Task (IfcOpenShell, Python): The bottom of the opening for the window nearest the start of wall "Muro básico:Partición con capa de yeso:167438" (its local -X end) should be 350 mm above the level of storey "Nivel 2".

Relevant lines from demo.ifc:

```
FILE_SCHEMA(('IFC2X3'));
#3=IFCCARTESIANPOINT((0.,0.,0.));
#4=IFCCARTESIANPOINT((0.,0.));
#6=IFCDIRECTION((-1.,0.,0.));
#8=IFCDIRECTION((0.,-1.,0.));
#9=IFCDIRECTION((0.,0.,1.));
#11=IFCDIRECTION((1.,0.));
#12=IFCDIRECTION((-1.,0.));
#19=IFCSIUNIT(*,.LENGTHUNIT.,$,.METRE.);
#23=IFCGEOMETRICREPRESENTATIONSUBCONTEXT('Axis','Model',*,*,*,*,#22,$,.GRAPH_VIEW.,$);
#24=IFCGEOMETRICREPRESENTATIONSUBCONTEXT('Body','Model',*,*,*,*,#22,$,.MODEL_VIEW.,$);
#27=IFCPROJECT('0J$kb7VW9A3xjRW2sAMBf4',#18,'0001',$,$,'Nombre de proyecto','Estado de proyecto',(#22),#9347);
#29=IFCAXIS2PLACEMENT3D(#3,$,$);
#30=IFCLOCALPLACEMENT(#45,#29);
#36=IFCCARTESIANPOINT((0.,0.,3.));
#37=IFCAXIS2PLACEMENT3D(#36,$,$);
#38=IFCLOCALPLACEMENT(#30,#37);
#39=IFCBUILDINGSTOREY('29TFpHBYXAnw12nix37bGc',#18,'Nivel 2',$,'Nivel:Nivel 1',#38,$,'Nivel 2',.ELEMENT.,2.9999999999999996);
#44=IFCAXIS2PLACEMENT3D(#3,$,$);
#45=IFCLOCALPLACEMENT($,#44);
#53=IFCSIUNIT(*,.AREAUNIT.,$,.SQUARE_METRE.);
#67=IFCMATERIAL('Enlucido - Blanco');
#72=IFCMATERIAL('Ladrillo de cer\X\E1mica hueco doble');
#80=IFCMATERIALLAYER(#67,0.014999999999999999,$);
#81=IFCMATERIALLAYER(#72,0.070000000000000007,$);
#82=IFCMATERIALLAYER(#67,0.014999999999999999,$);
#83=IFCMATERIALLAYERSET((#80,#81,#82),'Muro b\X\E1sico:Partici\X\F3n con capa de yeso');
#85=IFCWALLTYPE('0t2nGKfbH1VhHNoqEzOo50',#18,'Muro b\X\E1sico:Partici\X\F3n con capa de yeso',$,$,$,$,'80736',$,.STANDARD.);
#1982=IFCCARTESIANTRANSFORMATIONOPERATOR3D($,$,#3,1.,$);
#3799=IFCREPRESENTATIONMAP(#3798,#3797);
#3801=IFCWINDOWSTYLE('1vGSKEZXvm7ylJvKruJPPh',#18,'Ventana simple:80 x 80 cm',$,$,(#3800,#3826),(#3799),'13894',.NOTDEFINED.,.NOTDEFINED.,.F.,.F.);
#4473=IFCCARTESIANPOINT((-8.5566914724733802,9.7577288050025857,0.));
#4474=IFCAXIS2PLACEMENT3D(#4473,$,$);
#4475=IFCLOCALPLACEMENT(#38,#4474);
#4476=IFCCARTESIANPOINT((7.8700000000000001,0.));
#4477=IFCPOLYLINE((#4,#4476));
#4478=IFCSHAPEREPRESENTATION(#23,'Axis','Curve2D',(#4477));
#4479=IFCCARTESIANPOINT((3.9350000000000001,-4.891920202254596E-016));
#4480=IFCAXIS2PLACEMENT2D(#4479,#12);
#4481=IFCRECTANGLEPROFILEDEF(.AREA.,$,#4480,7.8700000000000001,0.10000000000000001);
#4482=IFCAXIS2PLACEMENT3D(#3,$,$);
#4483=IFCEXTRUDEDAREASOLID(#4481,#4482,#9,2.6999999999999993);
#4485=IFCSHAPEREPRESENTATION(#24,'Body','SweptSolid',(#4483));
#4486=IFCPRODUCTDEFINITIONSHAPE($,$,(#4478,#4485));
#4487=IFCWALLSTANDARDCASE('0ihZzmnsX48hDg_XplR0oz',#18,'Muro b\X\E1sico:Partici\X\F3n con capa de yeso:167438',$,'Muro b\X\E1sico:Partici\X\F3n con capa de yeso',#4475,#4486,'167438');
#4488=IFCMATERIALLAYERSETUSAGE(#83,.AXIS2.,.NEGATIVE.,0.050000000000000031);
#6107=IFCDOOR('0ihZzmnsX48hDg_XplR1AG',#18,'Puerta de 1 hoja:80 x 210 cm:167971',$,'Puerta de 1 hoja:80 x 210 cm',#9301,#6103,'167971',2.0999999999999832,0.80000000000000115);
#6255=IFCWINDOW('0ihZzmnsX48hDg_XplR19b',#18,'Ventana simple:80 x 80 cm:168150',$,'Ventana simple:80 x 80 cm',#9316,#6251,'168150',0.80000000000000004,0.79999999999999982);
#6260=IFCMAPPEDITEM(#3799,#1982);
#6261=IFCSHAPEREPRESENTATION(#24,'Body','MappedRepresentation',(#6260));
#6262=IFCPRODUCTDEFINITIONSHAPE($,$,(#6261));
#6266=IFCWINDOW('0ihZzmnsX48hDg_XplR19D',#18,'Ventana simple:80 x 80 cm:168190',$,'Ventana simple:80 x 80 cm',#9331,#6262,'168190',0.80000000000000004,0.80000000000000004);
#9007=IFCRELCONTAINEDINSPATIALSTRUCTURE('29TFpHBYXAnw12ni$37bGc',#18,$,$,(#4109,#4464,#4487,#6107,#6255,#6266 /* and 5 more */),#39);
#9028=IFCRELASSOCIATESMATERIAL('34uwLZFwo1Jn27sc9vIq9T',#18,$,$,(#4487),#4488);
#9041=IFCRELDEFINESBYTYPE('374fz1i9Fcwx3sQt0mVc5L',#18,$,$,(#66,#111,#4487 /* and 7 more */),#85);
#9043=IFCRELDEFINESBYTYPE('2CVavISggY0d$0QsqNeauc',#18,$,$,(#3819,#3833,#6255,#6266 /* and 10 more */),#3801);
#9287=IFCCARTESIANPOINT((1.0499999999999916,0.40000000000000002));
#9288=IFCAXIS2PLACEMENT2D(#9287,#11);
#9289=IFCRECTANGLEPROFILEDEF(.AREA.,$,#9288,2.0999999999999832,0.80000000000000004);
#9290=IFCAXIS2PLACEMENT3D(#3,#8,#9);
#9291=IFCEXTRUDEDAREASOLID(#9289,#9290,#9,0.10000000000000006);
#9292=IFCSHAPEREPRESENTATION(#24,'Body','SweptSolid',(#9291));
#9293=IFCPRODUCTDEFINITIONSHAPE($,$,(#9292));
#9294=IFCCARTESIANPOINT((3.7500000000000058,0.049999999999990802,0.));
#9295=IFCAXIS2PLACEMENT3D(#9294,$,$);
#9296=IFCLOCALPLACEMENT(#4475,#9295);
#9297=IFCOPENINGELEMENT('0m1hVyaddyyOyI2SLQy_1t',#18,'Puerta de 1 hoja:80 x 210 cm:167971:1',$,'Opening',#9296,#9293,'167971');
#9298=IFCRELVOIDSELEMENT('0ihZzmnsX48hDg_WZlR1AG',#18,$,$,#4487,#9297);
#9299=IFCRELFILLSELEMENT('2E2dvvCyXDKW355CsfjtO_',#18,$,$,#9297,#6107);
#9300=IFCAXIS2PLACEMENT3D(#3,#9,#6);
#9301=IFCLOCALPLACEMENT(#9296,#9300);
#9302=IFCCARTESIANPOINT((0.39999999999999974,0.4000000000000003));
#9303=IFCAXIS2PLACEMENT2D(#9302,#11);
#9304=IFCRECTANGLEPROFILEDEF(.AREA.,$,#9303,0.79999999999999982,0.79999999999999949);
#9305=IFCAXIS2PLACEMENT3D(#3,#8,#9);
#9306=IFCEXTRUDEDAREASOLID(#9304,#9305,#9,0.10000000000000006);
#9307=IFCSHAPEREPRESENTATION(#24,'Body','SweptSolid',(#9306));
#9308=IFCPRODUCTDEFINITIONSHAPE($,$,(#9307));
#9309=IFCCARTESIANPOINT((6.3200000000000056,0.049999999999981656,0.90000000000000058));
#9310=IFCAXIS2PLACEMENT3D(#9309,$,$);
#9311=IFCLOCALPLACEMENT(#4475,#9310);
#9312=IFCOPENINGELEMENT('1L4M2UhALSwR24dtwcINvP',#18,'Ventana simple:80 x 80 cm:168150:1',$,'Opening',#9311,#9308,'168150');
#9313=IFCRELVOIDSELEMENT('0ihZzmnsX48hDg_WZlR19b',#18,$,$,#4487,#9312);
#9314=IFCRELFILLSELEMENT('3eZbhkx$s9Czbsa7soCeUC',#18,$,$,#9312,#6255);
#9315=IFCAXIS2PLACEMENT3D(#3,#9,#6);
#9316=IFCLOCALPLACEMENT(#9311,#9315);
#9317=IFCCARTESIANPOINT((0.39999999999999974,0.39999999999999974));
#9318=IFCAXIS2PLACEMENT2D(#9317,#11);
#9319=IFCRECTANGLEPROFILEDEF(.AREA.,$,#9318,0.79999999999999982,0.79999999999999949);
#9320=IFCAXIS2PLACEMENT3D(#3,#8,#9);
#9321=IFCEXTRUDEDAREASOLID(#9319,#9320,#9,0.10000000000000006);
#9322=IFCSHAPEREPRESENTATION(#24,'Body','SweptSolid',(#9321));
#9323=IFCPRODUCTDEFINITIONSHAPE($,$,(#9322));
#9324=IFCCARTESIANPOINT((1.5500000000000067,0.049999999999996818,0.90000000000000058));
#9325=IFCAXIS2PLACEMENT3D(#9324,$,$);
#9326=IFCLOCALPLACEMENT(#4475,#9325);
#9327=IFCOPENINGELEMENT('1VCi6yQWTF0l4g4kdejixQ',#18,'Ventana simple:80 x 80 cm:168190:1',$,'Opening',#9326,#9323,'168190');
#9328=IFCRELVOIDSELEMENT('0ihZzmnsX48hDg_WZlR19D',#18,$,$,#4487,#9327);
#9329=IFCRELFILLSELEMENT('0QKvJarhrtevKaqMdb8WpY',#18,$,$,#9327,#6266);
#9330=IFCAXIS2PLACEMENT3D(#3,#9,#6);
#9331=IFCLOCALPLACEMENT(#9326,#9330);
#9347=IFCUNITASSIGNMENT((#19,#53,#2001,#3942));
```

```python
import numpy as np
import ifcopenshell
import ifcopenshell.api.geometry
import ifcopenshell.geom
import ifcopenshell.util.element
import ifcopenshell.util.placement
import ifcopenshell.util.shape
import ifcopenshell.util.unit

model = ifcopenshell.open("demo.ifc")
unit_scale = ifcopenshell.util.unit.calculate_unit_scale(model)

window = model.by_id(6266)
opening = window.FillsVoids[0].RelatingOpeningElement
storey = ifcopenshell.util.element.get_container(window, ifc_class="IfcBuildingStorey")
level = ifcopenshell.util.placement.get_local_placement(storey.ObjectPlacement)[2, 3]

# The opening's origin need not be at the sill, so measure its lowest point.
shape = ifcopenshell.geom.create_shape(ifcopenshell.geom.settings(), opening)
bottom = ifcopenshell.util.shape.get_shape_bottom_elevation(shape, shape.geometry) / unit_scale
dz = level + 0.35 / unit_scale - bottom

shift = np.array([0.0, 0.0, dz])
# The window is placed relative to its opening, so it follows when the opening moves.
matrix = ifcopenshell.util.placement.get_local_placement(opening.ObjectPlacement)
matrix[:3, 3] += shift
ifcopenshell.api.geometry.edit_object_placement(
    model, product=opening, matrix=matrix, is_si=False, should_transform_children=True
)

print(f"moved by {dz * unit_scale:+.3f} m")

model.write("demo-out.ifc")
```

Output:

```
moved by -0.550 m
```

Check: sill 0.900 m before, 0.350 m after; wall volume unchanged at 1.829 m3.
